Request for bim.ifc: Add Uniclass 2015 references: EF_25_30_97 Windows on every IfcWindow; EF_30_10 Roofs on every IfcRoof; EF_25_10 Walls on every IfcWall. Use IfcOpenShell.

First a look at what the model holds.

```python
import ifcopenshell

model = ifcopenshell.open("bim.ifc")
print(model.schema)
print("classifications:", [c.Name for c in model.by_type("IfcClassification")])
for ifc_class in ("IfcDoor", "IfcRoof", "IfcStair", "IfcWall", "IfcWindow"):
    print(ifc_class, len(model.by_type(ifc_class)))
```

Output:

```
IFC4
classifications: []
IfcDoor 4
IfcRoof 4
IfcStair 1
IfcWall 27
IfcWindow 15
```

```python
import ifcopenshell
import ifcopenshell.api.classification

model = ifcopenshell.open("bim.ifc")

system = ifcopenshell.api.classification.add_classification(model, classification="Uniclass 2015")

codes = {
    "IfcWindow": ("EF_25_30_97", "Windows"),
    "IfcRoof": ("EF_30_10", "Roofs"),
    "IfcWall": ("EF_25_10", "Walls"),
}
for ifc_class, (code, name) in codes.items():
    products = model.by_type(ifc_class)
    ifcopenshell.api.classification.add_reference(
        model, products=products, classification=system, identification=code, name=name
    )
    print(code, len(products))

model.write("bim_rev.ifc")
```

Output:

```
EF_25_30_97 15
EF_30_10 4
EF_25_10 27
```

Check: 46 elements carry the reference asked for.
